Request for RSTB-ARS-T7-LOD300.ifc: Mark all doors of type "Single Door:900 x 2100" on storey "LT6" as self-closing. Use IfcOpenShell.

First a look at what the model holds.

```python
import ifcopenshell
import ifcopenshell.util.element

model = ifcopenshell.open("RSTB-ARS-T7-LOD300.ifc")
print(model.schema)
storey = next(s for s in model.by_type("IfcBuildingStorey") if s.Name == "LT6")
doors = [e for e in ifcopenshell.util.element.get_decomposition(storey) if e.is_a("IfcDoor")]
seen = {}
for e in doors:
    element_type = ifcopenshell.util.element.get_type(e)
    key = (element_type.Name if element_type != e and element_type else None, ifcopenshell.util.element.get_pset(e, "Pset_DoorCommon", "SelfClosing"))
    seen[key] = seen.get(key, 0) + 1
for (name, value), count in sorted(seen.items(), key=str):
    print(count, "x", name, "|", value)
```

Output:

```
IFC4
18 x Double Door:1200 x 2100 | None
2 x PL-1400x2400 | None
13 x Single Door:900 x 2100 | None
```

```python
import ifcopenshell
import ifcopenshell.api.pset
import ifcopenshell.util.element

model = ifcopenshell.open("RSTB-ARS-T7-LOD300.ifc")

storey = next(s for s in model.by_type("IfcBuildingStorey") if s.Name == "LT6")
doors = [e for e in ifcopenshell.util.element.get_decomposition(storey) if e.is_a("IfcDoor")]

count = 0
for e in doors:
    element_type = ifcopenshell.util.element.get_type(e)
    if element_type in (None, e) or element_type.Name != "Single Door:900 x 2100":
        continue
    # add_pset returns the element's existing set when there is one.
    pset = ifcopenshell.api.pset.add_pset(model, product=e, name="Pset_DoorCommon")
    ifcopenshell.api.pset.edit_pset(model, pset=pset, properties={"SelfClosing": True})
    count += 1

print(count, "doors updated")

model.write("RSTB-ARS-T7-LOD300_rev.ifc")
```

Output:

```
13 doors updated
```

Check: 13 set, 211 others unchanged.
